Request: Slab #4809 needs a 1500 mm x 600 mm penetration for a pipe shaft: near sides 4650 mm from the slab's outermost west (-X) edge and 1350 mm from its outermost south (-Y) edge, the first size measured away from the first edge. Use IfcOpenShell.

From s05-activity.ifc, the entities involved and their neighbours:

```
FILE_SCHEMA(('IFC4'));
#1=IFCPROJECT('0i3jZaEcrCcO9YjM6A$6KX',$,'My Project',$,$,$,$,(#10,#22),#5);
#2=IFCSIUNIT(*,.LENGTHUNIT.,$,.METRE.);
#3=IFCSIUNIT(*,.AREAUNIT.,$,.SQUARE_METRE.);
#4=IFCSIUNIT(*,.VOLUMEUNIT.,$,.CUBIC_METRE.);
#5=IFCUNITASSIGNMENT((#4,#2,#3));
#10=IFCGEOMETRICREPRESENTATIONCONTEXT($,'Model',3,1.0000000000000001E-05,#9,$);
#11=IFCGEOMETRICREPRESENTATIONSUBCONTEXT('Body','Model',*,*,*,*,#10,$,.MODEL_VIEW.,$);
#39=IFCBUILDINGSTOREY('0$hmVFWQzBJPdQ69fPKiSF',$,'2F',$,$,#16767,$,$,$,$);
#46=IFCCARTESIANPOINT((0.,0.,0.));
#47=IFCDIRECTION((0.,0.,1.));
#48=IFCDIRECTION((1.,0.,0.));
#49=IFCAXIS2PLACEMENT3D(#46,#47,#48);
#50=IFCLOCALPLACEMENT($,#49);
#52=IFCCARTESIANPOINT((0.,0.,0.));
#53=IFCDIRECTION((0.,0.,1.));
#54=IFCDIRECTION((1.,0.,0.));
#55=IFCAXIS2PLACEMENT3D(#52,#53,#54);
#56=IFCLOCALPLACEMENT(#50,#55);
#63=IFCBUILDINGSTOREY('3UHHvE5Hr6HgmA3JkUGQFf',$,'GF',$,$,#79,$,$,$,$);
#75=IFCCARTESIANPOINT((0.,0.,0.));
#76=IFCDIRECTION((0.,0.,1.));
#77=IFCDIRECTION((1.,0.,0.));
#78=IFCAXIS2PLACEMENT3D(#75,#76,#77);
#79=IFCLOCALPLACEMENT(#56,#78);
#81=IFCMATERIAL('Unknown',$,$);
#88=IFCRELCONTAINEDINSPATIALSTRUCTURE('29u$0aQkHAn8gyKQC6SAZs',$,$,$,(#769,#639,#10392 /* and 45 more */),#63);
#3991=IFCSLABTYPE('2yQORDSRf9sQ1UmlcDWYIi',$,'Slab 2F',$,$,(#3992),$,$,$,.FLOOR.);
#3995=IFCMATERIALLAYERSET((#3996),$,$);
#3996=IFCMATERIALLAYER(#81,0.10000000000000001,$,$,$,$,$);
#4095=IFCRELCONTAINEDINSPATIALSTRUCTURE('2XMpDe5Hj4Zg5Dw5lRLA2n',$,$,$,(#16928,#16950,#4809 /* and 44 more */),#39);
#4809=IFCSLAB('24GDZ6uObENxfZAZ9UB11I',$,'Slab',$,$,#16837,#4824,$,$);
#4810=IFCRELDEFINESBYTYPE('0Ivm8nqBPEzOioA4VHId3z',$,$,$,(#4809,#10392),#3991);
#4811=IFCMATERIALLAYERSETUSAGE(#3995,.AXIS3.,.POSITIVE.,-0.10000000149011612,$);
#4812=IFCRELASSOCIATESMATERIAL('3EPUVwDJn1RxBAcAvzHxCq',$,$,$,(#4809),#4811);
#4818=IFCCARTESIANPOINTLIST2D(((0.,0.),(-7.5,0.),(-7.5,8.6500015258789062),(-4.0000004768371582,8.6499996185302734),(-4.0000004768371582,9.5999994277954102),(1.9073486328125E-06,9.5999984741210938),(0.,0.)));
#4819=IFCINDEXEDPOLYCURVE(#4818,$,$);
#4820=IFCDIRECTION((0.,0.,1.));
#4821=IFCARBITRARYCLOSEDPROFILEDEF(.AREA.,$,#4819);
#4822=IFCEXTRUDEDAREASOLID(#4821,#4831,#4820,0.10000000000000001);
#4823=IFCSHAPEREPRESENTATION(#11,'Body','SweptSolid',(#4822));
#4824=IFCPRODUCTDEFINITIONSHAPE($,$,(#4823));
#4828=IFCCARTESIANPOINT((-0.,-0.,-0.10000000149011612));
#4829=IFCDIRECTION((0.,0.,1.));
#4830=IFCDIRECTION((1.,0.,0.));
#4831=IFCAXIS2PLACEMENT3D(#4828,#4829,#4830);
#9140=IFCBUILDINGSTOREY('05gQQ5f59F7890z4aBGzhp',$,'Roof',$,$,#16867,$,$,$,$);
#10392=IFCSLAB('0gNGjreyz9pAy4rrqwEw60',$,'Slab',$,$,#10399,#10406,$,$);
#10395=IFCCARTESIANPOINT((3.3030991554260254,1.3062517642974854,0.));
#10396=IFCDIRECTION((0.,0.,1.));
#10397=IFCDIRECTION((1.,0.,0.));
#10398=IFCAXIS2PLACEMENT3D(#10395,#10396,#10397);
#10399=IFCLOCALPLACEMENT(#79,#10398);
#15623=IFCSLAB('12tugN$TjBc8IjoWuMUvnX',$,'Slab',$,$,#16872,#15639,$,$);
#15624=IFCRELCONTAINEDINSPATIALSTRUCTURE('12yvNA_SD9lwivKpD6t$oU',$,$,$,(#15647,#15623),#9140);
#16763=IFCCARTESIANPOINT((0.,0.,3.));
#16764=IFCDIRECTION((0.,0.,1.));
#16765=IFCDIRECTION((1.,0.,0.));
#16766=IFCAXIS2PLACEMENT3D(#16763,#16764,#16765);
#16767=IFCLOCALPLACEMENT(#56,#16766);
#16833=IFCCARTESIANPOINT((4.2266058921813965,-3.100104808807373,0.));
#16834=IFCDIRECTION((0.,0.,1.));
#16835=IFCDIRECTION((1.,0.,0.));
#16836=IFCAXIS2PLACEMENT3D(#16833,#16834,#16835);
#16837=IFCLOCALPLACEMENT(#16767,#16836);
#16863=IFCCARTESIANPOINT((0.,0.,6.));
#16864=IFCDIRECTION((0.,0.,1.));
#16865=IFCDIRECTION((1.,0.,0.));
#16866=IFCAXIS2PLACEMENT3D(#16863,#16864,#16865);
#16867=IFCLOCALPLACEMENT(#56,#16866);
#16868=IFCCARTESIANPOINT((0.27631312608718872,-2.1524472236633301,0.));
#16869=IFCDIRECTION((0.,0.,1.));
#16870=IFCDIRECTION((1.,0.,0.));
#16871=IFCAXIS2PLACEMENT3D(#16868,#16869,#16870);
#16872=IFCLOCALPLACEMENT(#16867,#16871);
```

```python
import numpy as np
import ifcopenshell
import ifcopenshell.api.feature
import ifcopenshell.api.geometry
import ifcopenshell.api.root
import ifcopenshell.geom
import ifcopenshell.util.placement
import ifcopenshell.util.representation
import ifcopenshell.util.shape
import ifcopenshell.util.unit

model = ifcopenshell.open("s05-activity.ifc")
unit_scale = ifcopenshell.util.unit.calculate_unit_scale(model)
settings = ifcopenshell.geom.settings()


def volume(element):
    """Net volume in cubic metres, openings subtracted."""
    shape = ifcopenshell.geom.create_shape(settings, element)
    return ifcopenshell.util.shape.get_volume(shape.geometry)


slab = model.by_guid("24GDZ6uObENxfZAZ9UB11I")
before = volume(slab)

# Extent in the slab's own axes, in metres. The edges named are its -X and -Y sides.
slab_shape = ifcopenshell.geom.create_shape(settings, slab)
vertices = ifcopenshell.util.shape.get_vertices(slab_shape.geometry)
x_min, y_min, bottom = vertices.min(axis=0)
top = vertices[:, 2].max()

opening = ifcopenshell.api.root.create_entity(model, ifc_class="IfcOpeningElement", name="Pipe shaft opening", predefined_type="OPENING")
context = ifcopenshell.util.representation.get_context(model, "Model", "Body", "MODEL_VIEW")
width, depth = 1.5, 0.6
outline = [(0.0, 0.0), (width, 0.0), (width, depth), (0.0, depth), (0.0, 0.0)]
# Overshoot both faces by 50 mm so the cut is clean.
shape = ifcopenshell.api.geometry.add_slab_representation(
    model, context=context, depth=top - bottom + 0.1, polyline=outline
)
ifcopenshell.api.geometry.assign_representation(model, product=opening, representation=shape)

matrix = ifcopenshell.util.placement.get_local_placement(slab.ObjectPlacement)
matrix[:, 3] = matrix @ np.append(np.array([x_min + 4.65, y_min + 1.35, bottom - 0.05]) / unit_scale, 1.0)
ifcopenshell.api.geometry.edit_object_placement(model, product=opening, matrix=matrix, is_si=False)
ifcopenshell.api.feature.add_feature(model, feature=opening, element=slab)

after = volume(slab)

print(f"slab volume {before:.3f} -> {after:.3f} m3")

model.write("s05-activity_edited.ifc")
```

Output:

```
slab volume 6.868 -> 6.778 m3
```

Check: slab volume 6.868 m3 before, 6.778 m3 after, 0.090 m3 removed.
